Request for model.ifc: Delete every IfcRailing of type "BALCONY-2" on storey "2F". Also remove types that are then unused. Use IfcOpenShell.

First a look at what the model holds.

```python
import ifcopenshell
import ifcopenshell.util.element

model = ifcopenshell.open("model.ifc")
print(model.schema)
storey = next(s for s in model.by_type("IfcBuildingStorey") if s.Name == "2F")
railings = [e for e in ifcopenshell.util.element.get_decomposition(storey) if e.is_a("IfcRailing")]
seen = {}
for e in railings:
    element_type = ifcopenshell.util.element.get_type(e)
    name = element_type.Name if element_type not in (None, e) else None
    seen[name] = seen.get(name, 0) + 1
for name, count in sorted(seen.items(), key=str):
    print(count, "x", name)
```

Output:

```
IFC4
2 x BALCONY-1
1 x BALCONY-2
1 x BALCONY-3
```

```python
import ifcopenshell
import ifcopenshell.api.root
import ifcopenshell.util.element

model = ifcopenshell.open("model.ifc")

storey = next(s for s in model.by_type("IfcBuildingStorey") if s.Name == "2F")
railings = [e for e in ifcopenshell.util.element.get_decomposition(storey) if e.is_a("IfcRailing")]
targets = [e for e in railings if (t := ifcopenshell.util.element.get_type(e)) not in (None, e) and t.Name == "BALCONY-2"]
types = {ifcopenshell.util.element.get_type(e) for e in targets} - {None, *targets}

for e in targets:
    ifcopenshell.api.root.remove_product(model, product=e)
print(len(targets), "removed")

unused = [t for t in types if not ifcopenshell.util.element.get_types(t)]
for t in unused:
    ifcopenshell.api.root.remove_product(model, product=t)
print(len(unused), "unused types removed")

model.write("model_rev.ifc")
```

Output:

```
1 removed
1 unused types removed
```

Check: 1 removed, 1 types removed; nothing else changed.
